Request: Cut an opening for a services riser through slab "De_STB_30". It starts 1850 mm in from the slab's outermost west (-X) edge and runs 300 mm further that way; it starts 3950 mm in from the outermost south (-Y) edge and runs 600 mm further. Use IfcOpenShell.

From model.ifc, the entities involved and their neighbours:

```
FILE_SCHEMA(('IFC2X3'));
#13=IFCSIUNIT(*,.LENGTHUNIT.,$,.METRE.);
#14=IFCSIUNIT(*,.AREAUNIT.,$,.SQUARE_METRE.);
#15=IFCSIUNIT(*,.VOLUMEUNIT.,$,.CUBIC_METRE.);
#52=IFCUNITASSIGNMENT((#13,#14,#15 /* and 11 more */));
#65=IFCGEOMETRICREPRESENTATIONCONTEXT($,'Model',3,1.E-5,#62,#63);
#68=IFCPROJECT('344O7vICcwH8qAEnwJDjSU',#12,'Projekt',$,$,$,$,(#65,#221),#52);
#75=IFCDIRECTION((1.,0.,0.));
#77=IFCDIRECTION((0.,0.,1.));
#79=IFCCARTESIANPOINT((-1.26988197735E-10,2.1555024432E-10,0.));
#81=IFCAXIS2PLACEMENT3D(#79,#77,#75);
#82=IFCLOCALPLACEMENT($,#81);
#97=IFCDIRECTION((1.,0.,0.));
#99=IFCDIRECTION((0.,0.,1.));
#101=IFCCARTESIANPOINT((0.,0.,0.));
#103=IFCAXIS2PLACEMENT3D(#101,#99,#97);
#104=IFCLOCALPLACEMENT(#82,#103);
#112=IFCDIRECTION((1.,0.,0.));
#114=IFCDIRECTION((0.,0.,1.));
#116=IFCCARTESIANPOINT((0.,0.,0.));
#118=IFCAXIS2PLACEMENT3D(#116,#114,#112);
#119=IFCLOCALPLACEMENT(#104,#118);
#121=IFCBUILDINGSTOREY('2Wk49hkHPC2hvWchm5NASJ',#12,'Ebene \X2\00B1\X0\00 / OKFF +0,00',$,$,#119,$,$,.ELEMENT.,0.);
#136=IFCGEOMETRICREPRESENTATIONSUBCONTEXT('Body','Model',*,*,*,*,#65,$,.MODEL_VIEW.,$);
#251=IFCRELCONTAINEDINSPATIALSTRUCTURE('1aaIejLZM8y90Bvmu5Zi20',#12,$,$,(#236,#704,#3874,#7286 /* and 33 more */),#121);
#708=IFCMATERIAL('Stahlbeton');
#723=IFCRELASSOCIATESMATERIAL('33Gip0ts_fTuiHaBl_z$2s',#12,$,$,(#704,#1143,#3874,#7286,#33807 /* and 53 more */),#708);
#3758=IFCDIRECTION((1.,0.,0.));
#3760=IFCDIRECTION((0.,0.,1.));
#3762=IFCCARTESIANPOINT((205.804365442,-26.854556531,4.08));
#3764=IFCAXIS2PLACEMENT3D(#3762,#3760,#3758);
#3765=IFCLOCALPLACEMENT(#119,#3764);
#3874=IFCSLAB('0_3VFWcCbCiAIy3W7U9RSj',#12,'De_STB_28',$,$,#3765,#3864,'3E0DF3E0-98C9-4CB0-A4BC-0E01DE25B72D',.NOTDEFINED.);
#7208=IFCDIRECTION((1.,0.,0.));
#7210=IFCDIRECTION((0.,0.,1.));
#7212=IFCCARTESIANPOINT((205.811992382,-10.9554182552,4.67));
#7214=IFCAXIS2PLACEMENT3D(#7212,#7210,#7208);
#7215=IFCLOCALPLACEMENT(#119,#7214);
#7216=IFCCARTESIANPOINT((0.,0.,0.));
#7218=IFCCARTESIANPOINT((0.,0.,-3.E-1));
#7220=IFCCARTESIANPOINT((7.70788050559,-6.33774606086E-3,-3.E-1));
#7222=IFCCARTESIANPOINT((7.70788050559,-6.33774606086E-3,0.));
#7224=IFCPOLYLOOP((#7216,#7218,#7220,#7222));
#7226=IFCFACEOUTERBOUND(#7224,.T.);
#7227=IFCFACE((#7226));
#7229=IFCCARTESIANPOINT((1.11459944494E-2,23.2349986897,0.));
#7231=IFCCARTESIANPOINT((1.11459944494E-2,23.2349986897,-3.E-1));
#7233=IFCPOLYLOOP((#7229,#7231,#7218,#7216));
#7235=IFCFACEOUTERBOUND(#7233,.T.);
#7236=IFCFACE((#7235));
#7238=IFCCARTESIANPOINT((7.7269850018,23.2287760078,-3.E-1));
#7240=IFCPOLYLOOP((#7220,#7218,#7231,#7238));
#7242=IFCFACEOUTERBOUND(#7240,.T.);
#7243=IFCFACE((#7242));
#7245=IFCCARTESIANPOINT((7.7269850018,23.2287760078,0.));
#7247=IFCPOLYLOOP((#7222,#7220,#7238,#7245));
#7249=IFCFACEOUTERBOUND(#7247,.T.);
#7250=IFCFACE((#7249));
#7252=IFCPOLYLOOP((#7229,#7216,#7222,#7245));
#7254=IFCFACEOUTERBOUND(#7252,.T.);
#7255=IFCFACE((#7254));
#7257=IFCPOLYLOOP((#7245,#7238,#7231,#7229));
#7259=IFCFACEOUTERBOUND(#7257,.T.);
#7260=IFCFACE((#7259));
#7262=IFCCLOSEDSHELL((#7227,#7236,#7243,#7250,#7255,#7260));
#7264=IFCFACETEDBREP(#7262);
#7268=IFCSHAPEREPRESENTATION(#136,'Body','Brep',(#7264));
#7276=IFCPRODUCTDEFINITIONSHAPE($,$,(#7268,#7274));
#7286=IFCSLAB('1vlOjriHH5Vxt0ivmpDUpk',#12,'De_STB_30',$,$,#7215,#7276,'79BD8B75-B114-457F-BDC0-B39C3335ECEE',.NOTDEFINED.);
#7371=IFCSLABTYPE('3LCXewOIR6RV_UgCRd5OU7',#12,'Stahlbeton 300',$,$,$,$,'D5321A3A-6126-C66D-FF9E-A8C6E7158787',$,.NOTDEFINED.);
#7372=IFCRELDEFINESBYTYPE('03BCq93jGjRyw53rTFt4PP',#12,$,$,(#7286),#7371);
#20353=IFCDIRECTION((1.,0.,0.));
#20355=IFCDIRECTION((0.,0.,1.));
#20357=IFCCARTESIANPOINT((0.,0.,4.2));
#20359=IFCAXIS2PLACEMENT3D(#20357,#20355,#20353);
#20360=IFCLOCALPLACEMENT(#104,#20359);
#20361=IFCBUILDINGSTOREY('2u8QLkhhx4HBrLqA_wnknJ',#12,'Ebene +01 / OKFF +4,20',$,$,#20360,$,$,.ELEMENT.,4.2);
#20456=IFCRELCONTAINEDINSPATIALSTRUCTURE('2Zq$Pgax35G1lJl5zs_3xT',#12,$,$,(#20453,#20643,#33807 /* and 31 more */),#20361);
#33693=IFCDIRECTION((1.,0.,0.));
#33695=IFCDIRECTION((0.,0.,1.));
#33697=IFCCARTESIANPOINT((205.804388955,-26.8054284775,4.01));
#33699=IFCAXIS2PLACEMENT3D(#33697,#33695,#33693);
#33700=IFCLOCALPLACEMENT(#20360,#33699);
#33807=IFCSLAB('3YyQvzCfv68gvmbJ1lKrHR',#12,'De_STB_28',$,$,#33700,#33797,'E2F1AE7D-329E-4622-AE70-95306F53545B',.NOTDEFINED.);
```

```python
import numpy as np
import ifcopenshell
import ifcopenshell.api.feature
import ifcopenshell.api.geometry
import ifcopenshell.api.root
import ifcopenshell.geom
import ifcopenshell.util.placement
import ifcopenshell.util.representation
import ifcopenshell.util.shape
import ifcopenshell.util.unit

model = ifcopenshell.open("model.ifc")
unit_scale = ifcopenshell.util.unit.calculate_unit_scale(model)
settings = ifcopenshell.geom.settings()


def volume(element):
    """Net volume in cubic metres, openings subtracted."""
    shape = ifcopenshell.geom.create_shape(settings, element)
    return ifcopenshell.util.shape.get_volume(shape.geometry)


slab = model.by_guid("1vlOjriHH5Vxt0ivmpDUpk")
before = volume(slab)

# Extent in the slab's own axes, in metres. The edges named are its -X and -Y sides.
slab_shape = ifcopenshell.geom.create_shape(settings, slab)
vertices = ifcopenshell.util.shape.get_vertices(slab_shape.geometry)
x_min, y_min, bottom = vertices.min(axis=0)
top = vertices[:, 2].max()

opening = ifcopenshell.api.root.create_entity(model, ifc_class="IfcOpeningElement", name="Services riser opening")
context = ifcopenshell.util.representation.get_context(model, "Model", "Body", "MODEL_VIEW")
width, depth = 0.3, 0.6
outline = [(0.0, 0.0), (width, 0.0), (width, depth), (0.0, depth), (0.0, 0.0)]
# Overshoot both faces by 50 mm so the cut is clean.
shape = ifcopenshell.api.geometry.add_slab_representation(
    model, context=context, depth=top - bottom + 0.1, polyline=outline
)
ifcopenshell.api.geometry.assign_representation(model, product=opening, representation=shape)

matrix = ifcopenshell.util.placement.get_local_placement(slab.ObjectPlacement)
matrix[:, 3] = matrix @ np.append(np.array([x_min + 1.85, y_min + 3.95, bottom - 0.05]) / unit_scale, 1.0)
ifcopenshell.api.geometry.edit_object_placement(model, product=opening, matrix=matrix, is_si=False)
ifcopenshell.api.feature.add_feature(model, feature=opening, element=slab)

after = volume(slab)

print(f"slab volume {before:.3f} -> {after:.3f} m3")

model.write("model_updated.ifc")
```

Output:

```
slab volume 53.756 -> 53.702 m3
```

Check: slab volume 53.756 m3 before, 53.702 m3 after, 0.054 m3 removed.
